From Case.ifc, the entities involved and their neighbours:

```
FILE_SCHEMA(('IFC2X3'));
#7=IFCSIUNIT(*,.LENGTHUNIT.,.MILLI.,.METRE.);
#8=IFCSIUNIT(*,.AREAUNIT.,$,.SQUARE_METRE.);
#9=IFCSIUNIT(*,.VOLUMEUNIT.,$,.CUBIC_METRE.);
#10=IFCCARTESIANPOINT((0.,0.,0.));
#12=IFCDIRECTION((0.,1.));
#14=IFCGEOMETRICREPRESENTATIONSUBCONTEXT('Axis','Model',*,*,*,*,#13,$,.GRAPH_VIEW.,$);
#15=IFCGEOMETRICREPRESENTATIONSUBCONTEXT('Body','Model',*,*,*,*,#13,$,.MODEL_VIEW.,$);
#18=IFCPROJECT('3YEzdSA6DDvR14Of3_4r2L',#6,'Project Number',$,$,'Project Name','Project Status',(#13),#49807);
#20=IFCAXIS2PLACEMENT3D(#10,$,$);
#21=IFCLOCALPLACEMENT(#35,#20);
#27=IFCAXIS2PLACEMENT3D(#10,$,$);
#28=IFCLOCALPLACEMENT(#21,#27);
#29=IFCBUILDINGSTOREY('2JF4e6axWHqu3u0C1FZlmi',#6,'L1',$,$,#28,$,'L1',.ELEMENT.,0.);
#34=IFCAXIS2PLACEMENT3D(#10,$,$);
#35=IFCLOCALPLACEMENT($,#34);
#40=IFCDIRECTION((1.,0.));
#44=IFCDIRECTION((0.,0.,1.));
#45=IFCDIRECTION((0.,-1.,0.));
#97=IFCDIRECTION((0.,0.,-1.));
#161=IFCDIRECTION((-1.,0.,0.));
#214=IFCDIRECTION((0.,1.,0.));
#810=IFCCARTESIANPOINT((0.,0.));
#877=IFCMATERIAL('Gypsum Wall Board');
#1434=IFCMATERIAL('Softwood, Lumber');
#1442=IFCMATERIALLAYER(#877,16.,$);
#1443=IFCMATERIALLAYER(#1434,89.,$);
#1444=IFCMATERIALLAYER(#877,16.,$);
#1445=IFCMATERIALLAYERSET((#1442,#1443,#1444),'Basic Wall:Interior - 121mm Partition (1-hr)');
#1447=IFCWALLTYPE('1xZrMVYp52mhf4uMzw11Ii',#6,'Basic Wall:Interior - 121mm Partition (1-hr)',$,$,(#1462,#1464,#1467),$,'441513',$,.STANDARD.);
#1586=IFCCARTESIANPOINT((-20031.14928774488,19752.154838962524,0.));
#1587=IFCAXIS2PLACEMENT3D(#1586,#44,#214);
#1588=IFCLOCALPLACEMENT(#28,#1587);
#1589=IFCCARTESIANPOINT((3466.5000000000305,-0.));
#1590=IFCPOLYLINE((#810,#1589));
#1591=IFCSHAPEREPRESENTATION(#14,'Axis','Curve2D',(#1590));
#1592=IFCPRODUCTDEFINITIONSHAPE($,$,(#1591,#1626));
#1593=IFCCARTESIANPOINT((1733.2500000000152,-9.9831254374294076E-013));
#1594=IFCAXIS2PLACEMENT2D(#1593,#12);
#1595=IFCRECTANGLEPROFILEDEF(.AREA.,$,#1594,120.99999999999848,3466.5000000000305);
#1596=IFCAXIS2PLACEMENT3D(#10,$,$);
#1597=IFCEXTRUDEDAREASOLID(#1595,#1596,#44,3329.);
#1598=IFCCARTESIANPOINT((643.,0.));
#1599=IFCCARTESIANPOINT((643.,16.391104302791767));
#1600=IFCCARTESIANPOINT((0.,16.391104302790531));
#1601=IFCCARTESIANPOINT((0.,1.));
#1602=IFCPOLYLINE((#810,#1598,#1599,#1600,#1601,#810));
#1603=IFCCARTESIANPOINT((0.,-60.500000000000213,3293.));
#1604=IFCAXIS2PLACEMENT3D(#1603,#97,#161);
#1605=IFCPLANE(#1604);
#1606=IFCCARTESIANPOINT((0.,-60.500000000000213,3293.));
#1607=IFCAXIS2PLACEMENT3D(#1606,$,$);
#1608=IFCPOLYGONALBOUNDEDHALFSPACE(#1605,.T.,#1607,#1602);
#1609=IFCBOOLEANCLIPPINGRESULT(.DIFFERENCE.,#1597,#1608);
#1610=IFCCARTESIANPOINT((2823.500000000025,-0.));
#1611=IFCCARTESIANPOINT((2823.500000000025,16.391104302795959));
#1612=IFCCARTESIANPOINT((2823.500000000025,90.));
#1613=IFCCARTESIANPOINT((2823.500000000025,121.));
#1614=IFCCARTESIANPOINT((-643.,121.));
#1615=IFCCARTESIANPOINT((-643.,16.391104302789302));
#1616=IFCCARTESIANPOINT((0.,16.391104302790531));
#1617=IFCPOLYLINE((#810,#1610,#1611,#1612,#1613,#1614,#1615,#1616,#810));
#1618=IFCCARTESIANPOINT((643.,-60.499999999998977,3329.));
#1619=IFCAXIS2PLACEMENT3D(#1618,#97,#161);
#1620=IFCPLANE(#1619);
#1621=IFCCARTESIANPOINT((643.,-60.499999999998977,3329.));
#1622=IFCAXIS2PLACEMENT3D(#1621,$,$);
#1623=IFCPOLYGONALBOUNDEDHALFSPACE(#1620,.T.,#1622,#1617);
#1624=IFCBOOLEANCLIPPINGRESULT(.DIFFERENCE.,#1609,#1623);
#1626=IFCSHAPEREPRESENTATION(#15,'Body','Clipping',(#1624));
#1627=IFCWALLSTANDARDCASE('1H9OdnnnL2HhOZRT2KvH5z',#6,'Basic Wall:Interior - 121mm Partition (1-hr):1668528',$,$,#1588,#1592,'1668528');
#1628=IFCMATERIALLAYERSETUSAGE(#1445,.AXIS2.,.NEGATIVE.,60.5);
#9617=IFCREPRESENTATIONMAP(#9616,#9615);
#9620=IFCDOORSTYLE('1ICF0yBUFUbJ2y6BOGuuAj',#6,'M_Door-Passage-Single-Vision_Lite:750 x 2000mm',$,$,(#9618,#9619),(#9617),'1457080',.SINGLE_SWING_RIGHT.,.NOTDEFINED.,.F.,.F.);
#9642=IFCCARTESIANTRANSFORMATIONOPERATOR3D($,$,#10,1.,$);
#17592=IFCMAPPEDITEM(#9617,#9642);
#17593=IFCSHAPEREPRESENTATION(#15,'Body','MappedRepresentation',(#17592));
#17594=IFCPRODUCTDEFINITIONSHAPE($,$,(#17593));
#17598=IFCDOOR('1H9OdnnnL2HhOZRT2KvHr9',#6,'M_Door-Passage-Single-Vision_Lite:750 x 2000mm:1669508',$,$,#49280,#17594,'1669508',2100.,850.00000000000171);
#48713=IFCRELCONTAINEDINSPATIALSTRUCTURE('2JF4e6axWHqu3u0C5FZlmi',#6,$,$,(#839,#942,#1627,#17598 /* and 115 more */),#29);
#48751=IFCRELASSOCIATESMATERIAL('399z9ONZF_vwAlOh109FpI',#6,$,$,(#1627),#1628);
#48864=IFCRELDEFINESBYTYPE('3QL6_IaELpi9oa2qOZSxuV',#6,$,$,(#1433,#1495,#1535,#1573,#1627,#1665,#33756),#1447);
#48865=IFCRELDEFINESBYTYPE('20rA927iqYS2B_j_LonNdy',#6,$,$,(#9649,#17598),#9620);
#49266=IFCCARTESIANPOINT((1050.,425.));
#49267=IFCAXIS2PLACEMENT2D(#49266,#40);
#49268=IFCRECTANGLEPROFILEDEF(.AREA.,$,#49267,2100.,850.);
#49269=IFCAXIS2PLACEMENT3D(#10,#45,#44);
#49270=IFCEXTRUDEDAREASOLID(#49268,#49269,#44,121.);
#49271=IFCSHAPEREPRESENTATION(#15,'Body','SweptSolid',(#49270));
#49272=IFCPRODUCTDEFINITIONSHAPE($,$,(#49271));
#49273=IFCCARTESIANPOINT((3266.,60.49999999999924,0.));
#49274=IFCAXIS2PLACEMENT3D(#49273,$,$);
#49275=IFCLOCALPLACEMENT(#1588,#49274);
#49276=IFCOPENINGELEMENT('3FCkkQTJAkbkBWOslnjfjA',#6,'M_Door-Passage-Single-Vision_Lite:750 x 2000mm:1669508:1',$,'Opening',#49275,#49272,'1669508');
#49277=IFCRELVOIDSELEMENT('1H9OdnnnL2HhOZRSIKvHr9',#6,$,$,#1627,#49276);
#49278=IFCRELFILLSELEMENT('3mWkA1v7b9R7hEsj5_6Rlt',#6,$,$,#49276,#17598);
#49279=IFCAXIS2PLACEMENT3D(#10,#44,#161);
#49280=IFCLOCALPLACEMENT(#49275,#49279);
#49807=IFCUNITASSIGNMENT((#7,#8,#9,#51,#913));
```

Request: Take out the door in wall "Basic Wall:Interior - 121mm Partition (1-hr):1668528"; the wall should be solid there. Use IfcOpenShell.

```python
import ifcopenshell
import ifcopenshell.api.feature
import ifcopenshell.api.root
import ifcopenshell.geom
import ifcopenshell.util.shape

model = ifcopenshell.open("Case.ifc")
settings = ifcopenshell.geom.settings()


def volume(element):
    """Net volume in cubic metres, openings subtracted."""
    shape = ifcopenshell.geom.create_shape(settings, element)
    return ifcopenshell.util.shape.get_volume(shape.geometry)


door = model.by_id(17598)
opening = door.FillsVoids[0].RelatingOpeningElement
wall = opening.VoidsElements[0].RelatingBuildingElement
before = volume(wall)

ifcopenshell.api.root.remove_product(model, product=door)
ifcopenshell.api.feature.remove_feature(model, feature=opening)

after = volume(wall)

print(f"wall volume {before:.3f} -> {after:.3f} m3")

model.write("Case-out.ifc")
```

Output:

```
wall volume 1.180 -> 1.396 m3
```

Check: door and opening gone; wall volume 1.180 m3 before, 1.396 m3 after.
